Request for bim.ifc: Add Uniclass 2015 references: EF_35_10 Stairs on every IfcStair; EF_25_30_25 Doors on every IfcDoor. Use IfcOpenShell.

First a look at what the model holds.

```python
import ifcopenshell

model = ifcopenshell.open("bim.ifc")
print(model.schema)
print("classifications:", [c.Name for c in model.by_type("IfcClassification")])
for ifc_class in ("IfcDoor", "IfcRoof", "IfcStair", "IfcWall", "IfcWindow"):
    print(ifc_class, len(model.by_type(ifc_class)))
```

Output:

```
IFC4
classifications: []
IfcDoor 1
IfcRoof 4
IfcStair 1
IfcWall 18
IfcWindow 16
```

```python
import ifcopenshell
import ifcopenshell.api.classification

model = ifcopenshell.open("bim.ifc")

system = ifcopenshell.api.classification.add_classification(model, classification="Uniclass 2015")

codes = {
    "IfcStair": ("EF_35_10", "Stairs"),
    "IfcDoor": ("EF_25_30_25", "Doors"),
}
for ifc_class, (code, name) in codes.items():
    products = model.by_type(ifc_class)
    ifcopenshell.api.classification.add_reference(
        model, products=products, classification=system, identification=code, name=name
    )
    print(code, len(products))

model.write("bim-out.ifc")
```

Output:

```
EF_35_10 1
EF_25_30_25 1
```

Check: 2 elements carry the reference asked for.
